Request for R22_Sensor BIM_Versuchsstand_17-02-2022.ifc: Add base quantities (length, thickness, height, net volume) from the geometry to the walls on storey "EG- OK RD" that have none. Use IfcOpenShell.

First a look at what the model holds.

```python
import ifcopenshell
import ifcopenshell.util.element
import ifcopenshell.util.unit

model = ifcopenshell.open("R22_Sensor BIM_Versuchsstand_17-02-2022.ifc")
print(model.schema)
for unit_type in ("LENGTHUNIT", "AREAUNIT", "VOLUMEUNIT"):
    print(unit_type, ifcopenshell.util.unit.calculate_unit_scale(model, unit_type))
storey = next(s for s in model.by_type("IfcBuildingStorey") if s.Name == "EG- OK RD")
walls = [e for e in ifcopenshell.util.element.get_decomposition(storey) if e.is_a("IfcWall")]
for e in sorted(walls, key=lambda e: e.id()):
    print(e.id(), e.is_a(), e.Name, list(ifcopenshell.util.element.get_psets(e, qtos_only=True)), sep=" | ")
```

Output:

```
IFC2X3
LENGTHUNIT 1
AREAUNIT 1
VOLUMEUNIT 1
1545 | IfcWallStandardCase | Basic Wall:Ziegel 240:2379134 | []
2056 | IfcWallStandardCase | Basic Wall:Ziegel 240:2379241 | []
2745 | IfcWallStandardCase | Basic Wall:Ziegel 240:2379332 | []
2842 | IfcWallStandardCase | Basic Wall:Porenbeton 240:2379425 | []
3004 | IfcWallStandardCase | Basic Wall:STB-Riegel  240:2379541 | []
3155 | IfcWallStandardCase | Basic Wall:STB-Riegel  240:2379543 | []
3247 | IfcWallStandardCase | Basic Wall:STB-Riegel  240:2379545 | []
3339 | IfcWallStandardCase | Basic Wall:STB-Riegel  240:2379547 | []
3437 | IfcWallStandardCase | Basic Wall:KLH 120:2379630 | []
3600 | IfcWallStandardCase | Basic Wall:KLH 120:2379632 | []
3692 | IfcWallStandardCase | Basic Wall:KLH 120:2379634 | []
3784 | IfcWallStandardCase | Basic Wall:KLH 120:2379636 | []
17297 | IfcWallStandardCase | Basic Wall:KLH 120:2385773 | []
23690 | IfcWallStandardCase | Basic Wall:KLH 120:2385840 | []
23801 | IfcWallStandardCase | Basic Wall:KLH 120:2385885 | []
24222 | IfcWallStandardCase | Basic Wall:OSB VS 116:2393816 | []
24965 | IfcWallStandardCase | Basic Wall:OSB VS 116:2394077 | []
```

```python
import ifcopenshell
import ifcopenshell.api.pset
import ifcopenshell.geom
import ifcopenshell.util.element
import ifcopenshell.util.shape
import ifcopenshell.util.unit

model = ifcopenshell.open("R22_Sensor BIM_Versuchsstand_17-02-2022.ifc")
unit_scale = ifcopenshell.util.unit.calculate_unit_scale(model)
volume_scale = ifcopenshell.util.unit.calculate_unit_scale(model, "VOLUMEUNIT")
settings = ifcopenshell.geom.settings()

storey = next(s for s in model.by_type("IfcBuildingStorey") if s.Name == "EG- OK RD")
walls = [e for e in ifcopenshell.util.element.get_decomposition(storey) if e.is_a("IfcWall")]

for e in sorted(walls, key=lambda e: e.id()):
    if ifcopenshell.util.element.get_psets(e, qtos_only=True, should_inherit=False):
        continue
    # Geometry comes back in metres, in the element's own axes.
    shape = ifcopenshell.geom.create_shape(settings, e)
    values = {
        "Length": ifcopenshell.util.shape.get_x(shape.geometry) / unit_scale,
        "Width": ifcopenshell.util.shape.get_y(shape.geometry) / unit_scale,
        "Height": ifcopenshell.util.shape.get_z(shape.geometry) / unit_scale,
        "NetVolume": ifcopenshell.util.shape.get_volume(shape.geometry) / volume_scale,
    }
    qto = ifcopenshell.api.pset.add_qto(model, product=e, name="BaseQuantities")
    ifcopenshell.api.pset.edit_qto(model, qto=qto, properties=values)
    print(e.id(), {k: round(v, 3) for k, v in values.items()})

model.write("R22_Sensor BIM_Versuchsstand_17-02-2022_rev.ifc")
```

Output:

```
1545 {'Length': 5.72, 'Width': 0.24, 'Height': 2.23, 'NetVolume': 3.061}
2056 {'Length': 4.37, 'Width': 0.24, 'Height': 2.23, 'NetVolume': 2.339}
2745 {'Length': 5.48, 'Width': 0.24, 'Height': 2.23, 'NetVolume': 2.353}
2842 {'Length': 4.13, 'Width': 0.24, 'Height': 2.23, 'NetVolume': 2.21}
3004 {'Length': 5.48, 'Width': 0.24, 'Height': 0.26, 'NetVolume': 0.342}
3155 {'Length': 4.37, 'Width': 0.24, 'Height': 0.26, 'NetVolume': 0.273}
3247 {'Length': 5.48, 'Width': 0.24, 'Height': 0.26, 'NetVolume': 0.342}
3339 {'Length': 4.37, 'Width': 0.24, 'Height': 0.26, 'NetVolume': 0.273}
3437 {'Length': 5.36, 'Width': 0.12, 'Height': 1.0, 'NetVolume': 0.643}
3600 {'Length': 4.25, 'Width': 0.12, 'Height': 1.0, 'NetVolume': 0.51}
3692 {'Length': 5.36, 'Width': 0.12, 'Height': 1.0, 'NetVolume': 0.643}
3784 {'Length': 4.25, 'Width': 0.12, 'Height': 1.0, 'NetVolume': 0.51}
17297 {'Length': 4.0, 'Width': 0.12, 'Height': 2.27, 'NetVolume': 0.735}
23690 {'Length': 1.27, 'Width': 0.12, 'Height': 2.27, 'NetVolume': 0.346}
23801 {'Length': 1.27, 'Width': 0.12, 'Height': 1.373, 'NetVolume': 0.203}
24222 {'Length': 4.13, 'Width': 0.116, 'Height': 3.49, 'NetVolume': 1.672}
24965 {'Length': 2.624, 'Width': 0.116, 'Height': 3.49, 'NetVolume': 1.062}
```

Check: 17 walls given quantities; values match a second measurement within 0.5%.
